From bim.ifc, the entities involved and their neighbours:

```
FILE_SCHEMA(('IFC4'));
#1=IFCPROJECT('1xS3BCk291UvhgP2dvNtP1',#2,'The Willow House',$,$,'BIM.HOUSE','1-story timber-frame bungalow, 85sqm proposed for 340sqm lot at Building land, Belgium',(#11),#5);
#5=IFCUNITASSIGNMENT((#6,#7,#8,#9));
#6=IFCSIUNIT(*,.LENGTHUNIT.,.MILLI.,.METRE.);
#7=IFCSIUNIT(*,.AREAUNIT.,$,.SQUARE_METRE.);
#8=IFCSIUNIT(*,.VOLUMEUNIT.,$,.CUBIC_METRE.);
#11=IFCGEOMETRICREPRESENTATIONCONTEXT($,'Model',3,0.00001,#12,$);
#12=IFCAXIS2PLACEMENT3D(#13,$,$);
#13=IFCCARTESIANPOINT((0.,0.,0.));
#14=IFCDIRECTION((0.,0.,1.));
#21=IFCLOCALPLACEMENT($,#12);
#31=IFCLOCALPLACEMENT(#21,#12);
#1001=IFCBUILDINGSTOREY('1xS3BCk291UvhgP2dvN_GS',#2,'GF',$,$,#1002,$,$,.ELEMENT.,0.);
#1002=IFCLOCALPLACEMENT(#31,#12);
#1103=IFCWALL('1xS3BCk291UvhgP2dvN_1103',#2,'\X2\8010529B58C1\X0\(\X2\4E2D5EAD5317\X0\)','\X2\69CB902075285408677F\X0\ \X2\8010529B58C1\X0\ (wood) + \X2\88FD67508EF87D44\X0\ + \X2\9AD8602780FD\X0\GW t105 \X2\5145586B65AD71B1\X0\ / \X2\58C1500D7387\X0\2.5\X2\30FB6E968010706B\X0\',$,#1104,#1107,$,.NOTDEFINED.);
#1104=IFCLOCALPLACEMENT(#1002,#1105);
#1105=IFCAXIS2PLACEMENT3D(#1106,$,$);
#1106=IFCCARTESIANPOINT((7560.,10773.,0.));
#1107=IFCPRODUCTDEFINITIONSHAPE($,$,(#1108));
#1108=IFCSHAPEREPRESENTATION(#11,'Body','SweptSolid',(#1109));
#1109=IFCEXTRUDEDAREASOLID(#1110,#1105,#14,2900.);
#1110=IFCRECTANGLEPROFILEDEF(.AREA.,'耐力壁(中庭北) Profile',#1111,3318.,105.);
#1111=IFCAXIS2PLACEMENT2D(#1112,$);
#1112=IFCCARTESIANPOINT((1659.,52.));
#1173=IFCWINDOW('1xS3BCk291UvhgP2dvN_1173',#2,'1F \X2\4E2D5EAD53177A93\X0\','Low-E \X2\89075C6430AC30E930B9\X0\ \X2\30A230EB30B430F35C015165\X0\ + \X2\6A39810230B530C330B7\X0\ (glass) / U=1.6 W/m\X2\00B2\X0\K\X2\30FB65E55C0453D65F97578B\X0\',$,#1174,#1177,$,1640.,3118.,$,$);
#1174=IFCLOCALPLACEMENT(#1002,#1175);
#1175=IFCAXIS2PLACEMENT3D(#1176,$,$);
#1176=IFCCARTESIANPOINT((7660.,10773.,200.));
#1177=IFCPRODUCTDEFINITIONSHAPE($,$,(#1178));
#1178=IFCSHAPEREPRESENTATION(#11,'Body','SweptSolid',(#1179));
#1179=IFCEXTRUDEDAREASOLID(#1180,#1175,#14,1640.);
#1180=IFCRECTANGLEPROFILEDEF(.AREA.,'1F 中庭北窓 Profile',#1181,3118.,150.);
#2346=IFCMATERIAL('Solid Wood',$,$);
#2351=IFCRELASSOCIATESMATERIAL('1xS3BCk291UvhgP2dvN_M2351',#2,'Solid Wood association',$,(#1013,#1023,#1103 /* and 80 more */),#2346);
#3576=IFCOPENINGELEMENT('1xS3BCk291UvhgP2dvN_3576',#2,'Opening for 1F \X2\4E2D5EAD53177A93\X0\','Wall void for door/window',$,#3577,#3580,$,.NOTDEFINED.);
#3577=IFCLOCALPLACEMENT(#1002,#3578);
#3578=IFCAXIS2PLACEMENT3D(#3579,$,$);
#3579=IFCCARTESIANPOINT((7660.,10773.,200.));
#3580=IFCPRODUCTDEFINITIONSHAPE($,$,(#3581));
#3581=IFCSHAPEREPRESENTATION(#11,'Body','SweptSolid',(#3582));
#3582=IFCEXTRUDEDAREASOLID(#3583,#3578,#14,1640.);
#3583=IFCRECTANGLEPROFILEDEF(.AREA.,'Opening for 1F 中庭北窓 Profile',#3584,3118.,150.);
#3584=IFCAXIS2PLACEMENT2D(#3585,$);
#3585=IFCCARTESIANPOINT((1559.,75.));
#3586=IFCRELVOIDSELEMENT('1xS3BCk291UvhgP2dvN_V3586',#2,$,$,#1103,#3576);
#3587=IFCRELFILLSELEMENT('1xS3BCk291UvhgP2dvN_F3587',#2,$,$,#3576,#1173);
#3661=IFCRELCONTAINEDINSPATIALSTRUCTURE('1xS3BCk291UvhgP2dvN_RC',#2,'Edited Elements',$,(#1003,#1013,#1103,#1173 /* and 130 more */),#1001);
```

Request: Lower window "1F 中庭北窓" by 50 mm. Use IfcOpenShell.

```python
import numpy as np
import ifcopenshell
import ifcopenshell.api.geometry
import ifcopenshell.util.placement
import ifcopenshell.util.unit

model = ifcopenshell.open("bim.ifc")
unit_scale = ifcopenshell.util.unit.calculate_unit_scale(model)

window = model.by_guid("1xS3BCk291UvhgP2dvN_1173")
opening = window.FillsVoids[0].RelatingOpeningElement
dz = -0.05 / unit_scale

shift = np.array([0.0, 0.0, dz])
# The window is not placed relative to its opening, so move both.
for product in (opening, window):
    matrix = ifcopenshell.util.placement.get_local_placement(product.ObjectPlacement)
    matrix[:3, 3] += shift
    ifcopenshell.api.geometry.edit_object_placement(model, product=product, matrix=matrix, is_si=False)

print(f"moved by {dz * unit_scale:+.3f} m")

model.write("bim_v2.ifc")
```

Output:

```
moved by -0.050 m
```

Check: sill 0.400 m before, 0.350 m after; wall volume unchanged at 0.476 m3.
